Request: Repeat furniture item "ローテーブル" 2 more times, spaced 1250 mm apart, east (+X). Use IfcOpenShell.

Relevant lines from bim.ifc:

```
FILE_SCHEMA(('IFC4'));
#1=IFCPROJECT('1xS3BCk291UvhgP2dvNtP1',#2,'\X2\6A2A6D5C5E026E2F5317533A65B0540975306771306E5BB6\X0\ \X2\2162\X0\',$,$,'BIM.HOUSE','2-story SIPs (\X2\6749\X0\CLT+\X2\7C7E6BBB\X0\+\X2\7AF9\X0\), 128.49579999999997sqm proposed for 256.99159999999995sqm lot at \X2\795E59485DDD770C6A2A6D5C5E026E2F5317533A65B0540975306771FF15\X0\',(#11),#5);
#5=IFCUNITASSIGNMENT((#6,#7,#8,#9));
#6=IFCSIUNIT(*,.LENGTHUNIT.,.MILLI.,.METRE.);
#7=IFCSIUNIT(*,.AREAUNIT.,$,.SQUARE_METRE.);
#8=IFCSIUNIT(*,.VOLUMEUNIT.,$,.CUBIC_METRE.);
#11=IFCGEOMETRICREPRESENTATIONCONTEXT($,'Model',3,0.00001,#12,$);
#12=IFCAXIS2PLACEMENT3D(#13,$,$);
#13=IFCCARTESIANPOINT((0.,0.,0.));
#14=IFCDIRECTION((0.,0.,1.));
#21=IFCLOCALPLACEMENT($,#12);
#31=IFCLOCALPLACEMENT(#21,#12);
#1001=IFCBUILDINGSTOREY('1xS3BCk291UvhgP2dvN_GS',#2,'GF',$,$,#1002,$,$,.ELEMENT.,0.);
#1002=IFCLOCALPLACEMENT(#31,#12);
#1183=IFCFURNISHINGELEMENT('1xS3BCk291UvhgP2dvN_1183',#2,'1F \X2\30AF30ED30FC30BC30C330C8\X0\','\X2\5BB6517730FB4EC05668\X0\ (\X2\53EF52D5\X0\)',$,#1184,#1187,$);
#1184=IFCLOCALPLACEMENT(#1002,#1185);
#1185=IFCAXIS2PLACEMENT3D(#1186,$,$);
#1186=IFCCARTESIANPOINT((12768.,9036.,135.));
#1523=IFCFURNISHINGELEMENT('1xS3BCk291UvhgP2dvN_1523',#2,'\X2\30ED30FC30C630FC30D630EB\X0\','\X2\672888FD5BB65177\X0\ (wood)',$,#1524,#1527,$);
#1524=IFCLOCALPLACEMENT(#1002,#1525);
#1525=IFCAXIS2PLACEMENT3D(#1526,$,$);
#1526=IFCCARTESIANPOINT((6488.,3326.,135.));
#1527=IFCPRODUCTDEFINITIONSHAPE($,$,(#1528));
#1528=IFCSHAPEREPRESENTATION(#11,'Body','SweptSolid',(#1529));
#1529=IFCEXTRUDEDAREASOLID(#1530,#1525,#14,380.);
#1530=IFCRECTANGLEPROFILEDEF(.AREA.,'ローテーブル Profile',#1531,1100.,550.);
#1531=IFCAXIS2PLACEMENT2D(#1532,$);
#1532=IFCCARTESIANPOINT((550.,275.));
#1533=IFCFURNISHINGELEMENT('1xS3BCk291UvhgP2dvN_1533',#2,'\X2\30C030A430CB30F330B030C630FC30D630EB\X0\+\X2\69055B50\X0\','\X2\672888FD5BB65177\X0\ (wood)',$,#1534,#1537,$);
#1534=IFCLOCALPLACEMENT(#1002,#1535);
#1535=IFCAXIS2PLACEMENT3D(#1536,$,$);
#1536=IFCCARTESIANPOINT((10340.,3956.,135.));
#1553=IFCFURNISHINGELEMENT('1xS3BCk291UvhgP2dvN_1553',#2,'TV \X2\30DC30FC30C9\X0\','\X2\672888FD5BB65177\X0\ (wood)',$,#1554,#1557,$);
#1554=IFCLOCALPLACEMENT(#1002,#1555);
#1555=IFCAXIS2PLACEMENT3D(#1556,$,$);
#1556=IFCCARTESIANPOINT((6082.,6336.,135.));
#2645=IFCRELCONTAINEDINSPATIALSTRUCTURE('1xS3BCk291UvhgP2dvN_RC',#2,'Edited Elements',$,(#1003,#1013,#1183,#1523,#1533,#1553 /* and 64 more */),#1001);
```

```python
import numpy as np
import ifcopenshell
import ifcopenshell.api.geometry
import ifcopenshell.api.root
import ifcopenshell.util.element
import ifcopenshell.util.placement

model = ifcopenshell.open("bim.ifc")


def reuse_history(source, copy):
    """copy_class also copies each property set's owner history, people and application; keep the originals."""
    for rel in copy.IsDefinedBy:
        if rel.is_a("IfcRelDefinesByProperties") and (history := rel.RelatingPropertyDefinition.OwnerHistory):
            rel.RelatingPropertyDefinition.OwnerHistory = source.OwnerHistory
            ifcopenshell.util.element.remove_deep2(model, history)


source = model.by_guid("1xS3BCk291UvhgP2dvN_1523")
base = ifcopenshell.util.placement.get_local_placement(source.ObjectPlacement)
step = np.array([1.0, 0.0, 0.0]) * 1250.0

for i in range(1, 3):
    copy = ifcopenshell.api.root.copy_class(model, product=source)
    copy.Representation = ifcopenshell.util.element.copy_deep(
        model, source.Representation, exclude=["IfcGeometricRepresentationContext", "IfcRepresentationMap"]
    )
    reuse_history(source, copy)
    matrix = base.copy()
    matrix[:3, 3] += i * step
    print("added at", matrix[:3, 3].round(3) + 0.0)
    ifcopenshell.api.geometry.edit_object_placement(model, product=copy, matrix=matrix, is_si=False)

model.write("bim_v2.ifc")
```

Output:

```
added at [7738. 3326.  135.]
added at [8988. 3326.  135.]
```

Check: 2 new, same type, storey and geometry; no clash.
